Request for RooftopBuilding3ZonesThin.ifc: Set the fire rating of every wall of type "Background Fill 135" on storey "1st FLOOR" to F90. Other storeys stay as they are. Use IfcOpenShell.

First a look at what the model holds.

```python
import ifcopenshell
import ifcopenshell.util.element

model = ifcopenshell.open("RooftopBuilding3ZonesThin.ifc")
print(model.schema)
storey = next(s for s in model.by_type("IfcBuildingStorey") if s.Name == "1st FLOOR")
walls = [e for e in ifcopenshell.util.element.get_decomposition(storey) if e.is_a("IfcWall")]
seen = {}
for e in walls:
    element_type = ifcopenshell.util.element.get_type(e)
    key = (element_type.Name if element_type != e and element_type else None, ifcopenshell.util.element.get_pset(e, "Pset_WallCommon", "FireRating"))
    seen[key] = seen.get(key, 0) + 1
for (name, value), count in sorted(seen.items(), key=str):
    print(count, "x", name, "|", value)
```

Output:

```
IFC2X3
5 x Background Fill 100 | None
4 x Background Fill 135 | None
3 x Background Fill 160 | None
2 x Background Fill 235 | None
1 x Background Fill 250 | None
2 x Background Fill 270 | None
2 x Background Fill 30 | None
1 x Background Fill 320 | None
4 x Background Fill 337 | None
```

```python
import ifcopenshell
import ifcopenshell.api.pset
import ifcopenshell.util.element

model = ifcopenshell.open("RooftopBuilding3ZonesThin.ifc")

storey = next(s for s in model.by_type("IfcBuildingStorey") if s.Name == "1st FLOOR")
walls = [e for e in ifcopenshell.util.element.get_decomposition(storey) if e.is_a("IfcWall")]

count = 0
for e in walls:
    element_type = ifcopenshell.util.element.get_type(e)
    if element_type in (None, e) or element_type.Name != "Background Fill 135":
        continue
    # add_pset returns the element's existing set when there is one.
    pset = ifcopenshell.api.pset.add_pset(model, product=e, name="Pset_WallCommon")
    ifcopenshell.api.pset.edit_pset(model, pset=pset, properties={"FireRating": "F90"})
    count += 1

print(count, "walls updated")

model.write("RooftopBuilding3ZonesThin_v2.ifc")
```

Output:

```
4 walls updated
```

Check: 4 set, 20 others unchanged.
